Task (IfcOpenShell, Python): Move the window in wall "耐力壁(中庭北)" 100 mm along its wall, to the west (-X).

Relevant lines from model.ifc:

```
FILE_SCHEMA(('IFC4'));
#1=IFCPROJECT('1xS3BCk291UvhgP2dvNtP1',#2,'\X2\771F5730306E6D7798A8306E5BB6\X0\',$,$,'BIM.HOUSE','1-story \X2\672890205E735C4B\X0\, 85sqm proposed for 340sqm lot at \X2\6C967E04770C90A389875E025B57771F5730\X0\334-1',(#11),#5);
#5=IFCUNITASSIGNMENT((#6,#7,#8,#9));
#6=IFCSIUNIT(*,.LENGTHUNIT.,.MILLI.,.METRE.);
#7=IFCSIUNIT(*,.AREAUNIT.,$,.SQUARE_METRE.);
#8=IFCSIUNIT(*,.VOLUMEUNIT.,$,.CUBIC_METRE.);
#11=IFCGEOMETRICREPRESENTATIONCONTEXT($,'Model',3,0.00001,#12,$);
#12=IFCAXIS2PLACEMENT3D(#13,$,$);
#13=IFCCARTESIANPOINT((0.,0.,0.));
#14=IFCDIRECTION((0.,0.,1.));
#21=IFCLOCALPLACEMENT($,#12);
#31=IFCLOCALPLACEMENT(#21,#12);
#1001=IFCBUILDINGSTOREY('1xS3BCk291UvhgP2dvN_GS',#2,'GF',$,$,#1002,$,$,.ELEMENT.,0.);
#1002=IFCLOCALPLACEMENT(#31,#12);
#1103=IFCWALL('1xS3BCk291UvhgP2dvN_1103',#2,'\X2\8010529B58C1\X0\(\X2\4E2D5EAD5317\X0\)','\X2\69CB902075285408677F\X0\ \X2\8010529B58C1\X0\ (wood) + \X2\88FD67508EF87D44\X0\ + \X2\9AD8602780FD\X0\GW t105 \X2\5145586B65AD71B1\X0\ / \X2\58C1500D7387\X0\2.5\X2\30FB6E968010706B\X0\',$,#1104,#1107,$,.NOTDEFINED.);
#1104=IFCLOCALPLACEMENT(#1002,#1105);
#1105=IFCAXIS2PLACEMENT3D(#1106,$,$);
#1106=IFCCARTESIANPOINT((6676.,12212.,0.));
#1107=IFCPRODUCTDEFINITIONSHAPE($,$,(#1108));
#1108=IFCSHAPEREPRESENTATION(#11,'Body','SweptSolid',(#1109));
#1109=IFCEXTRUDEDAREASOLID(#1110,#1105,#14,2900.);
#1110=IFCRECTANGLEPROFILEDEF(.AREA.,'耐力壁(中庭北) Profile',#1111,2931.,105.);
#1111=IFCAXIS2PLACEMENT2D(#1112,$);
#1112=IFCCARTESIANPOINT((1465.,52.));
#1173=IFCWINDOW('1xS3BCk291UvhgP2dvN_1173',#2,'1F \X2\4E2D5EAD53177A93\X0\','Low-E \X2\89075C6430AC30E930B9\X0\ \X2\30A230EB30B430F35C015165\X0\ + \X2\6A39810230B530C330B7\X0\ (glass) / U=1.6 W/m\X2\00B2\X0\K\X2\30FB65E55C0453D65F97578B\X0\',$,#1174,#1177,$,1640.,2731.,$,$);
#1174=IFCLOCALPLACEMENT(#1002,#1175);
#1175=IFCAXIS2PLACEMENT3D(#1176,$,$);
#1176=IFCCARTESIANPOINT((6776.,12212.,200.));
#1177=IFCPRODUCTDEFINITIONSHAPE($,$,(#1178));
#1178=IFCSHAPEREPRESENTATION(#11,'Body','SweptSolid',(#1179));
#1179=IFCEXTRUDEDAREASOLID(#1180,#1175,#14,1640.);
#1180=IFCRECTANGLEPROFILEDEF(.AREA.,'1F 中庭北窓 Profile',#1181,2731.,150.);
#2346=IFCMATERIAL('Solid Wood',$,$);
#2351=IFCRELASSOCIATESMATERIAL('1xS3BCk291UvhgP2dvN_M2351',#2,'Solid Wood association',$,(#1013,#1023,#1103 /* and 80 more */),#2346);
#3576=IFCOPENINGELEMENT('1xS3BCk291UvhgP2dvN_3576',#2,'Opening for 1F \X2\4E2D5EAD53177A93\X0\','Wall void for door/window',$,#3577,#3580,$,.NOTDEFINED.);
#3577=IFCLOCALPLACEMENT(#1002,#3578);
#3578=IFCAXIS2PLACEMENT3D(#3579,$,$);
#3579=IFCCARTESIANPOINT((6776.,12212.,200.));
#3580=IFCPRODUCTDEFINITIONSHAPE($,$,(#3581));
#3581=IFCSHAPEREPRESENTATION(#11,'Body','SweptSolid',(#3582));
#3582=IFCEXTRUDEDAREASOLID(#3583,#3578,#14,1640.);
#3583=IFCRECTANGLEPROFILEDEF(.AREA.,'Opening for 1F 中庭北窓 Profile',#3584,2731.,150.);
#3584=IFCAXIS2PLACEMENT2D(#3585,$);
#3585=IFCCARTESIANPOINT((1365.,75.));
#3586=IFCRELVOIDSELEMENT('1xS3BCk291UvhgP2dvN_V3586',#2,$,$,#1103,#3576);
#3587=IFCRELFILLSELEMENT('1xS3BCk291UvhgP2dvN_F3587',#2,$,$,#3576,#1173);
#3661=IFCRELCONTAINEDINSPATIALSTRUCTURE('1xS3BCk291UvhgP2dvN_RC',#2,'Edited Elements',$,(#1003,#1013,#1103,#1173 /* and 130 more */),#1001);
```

```python
import ifcopenshell
import ifcopenshell.api.geometry
import ifcopenshell.util.placement

model = ifcopenshell.open("model.ifc")

window = model.by_guid("1xS3BCk291UvhgP2dvN_1173")
opening = window.FillsVoids[0].RelatingOpeningElement
wall = opening.VoidsElements[0].RelatingBuildingElement

wall_matrix = ifcopenshell.util.placement.get_local_placement(wall.ObjectPlacement)
shift = wall_matrix[:3, 0] * -100.0
before = ifcopenshell.util.placement.get_local_placement(window.ObjectPlacement)[:3, 3].copy()

# The window is not placed relative to its opening, so move both.
for product in (opening, window):
    matrix = ifcopenshell.util.placement.get_local_placement(product.ObjectPlacement)
    matrix[:3, 3] += shift
    ifcopenshell.api.geometry.edit_object_placement(model, product=product, matrix=matrix, is_si=False)

after = ifcopenshell.util.placement.get_local_placement(window.ObjectPlacement)[:3, 3]
print("window moved by", (after - before).round(3) + 0.0)

model.write("model_v2.ifc")
```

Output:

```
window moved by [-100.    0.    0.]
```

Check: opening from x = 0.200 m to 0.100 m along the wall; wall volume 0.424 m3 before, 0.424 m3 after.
